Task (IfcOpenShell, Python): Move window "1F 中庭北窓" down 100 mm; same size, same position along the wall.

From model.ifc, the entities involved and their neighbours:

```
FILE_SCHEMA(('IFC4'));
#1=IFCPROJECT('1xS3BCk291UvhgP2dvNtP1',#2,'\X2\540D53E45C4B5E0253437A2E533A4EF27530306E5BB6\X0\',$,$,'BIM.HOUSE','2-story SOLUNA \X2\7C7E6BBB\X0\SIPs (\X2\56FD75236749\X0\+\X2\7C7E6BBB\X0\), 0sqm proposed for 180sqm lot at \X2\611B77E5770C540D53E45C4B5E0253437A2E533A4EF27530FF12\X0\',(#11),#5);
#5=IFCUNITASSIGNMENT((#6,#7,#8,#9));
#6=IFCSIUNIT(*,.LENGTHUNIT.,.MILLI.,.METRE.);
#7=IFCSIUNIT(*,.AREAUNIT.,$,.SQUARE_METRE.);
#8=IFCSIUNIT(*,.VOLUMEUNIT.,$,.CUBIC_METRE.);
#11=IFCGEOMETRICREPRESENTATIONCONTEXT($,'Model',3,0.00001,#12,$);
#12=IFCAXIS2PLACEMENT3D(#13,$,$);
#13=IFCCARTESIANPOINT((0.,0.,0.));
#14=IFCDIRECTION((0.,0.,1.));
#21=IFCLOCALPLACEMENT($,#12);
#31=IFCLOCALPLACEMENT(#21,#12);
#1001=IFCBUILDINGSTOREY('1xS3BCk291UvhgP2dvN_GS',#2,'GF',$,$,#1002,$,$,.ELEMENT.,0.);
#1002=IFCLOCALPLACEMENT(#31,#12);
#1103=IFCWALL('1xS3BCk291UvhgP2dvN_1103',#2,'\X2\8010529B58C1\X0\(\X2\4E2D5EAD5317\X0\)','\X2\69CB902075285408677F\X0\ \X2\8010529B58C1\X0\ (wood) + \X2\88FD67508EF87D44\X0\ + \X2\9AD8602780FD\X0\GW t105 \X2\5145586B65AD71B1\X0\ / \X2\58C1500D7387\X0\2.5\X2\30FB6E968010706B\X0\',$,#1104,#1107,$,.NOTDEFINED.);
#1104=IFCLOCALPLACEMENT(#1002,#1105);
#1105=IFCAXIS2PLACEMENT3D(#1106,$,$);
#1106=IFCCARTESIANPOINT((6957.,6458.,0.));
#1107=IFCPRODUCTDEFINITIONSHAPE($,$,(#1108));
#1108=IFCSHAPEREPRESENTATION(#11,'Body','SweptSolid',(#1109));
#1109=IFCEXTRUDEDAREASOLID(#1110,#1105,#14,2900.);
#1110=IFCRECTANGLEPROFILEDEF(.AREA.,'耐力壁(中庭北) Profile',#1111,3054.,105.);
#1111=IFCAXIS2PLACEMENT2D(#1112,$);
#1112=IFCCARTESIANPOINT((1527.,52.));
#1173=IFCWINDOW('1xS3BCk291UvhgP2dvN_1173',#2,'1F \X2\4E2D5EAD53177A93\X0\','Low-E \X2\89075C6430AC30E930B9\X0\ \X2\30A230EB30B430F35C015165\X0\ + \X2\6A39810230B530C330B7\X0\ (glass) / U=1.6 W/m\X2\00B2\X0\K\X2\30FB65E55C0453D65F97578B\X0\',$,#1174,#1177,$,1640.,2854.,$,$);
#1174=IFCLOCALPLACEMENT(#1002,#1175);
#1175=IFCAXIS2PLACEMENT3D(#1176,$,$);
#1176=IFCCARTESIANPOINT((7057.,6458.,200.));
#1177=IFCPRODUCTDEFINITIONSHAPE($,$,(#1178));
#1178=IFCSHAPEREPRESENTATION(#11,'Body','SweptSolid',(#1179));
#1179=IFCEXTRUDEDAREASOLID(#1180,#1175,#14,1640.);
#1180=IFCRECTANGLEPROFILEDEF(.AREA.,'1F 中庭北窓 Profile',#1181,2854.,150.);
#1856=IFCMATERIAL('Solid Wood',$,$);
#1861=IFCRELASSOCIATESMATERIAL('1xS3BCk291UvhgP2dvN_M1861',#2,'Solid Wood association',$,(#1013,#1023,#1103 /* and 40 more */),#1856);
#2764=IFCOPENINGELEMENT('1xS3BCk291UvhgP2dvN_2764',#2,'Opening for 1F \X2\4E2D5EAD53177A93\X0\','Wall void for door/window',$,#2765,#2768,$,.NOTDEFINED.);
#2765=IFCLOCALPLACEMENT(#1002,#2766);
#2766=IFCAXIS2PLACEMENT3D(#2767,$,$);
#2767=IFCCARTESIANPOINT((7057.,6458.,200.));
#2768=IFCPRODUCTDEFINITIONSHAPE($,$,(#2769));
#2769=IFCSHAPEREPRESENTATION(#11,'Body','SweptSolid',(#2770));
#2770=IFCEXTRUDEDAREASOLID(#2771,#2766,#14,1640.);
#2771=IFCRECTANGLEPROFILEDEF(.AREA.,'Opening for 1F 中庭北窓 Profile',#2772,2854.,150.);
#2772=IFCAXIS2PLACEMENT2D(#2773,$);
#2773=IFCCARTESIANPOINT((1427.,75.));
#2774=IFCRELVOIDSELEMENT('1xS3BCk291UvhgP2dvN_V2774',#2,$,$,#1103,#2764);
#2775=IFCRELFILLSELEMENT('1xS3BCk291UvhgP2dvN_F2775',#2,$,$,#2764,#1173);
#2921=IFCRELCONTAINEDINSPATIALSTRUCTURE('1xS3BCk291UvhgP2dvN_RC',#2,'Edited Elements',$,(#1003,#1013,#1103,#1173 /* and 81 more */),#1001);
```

```python
import numpy as np
import ifcopenshell
import ifcopenshell.api.geometry
import ifcopenshell.util.placement
import ifcopenshell.util.unit

model = ifcopenshell.open("model.ifc")
unit_scale = ifcopenshell.util.unit.calculate_unit_scale(model)

window = model.by_guid("1xS3BCk291UvhgP2dvN_1173")
opening = window.FillsVoids[0].RelatingOpeningElement
dz = -0.1 / unit_scale

shift = np.array([0.0, 0.0, dz])
# The window is not placed relative to its opening, so move both.
for product in (opening, window):
    matrix = ifcopenshell.util.placement.get_local_placement(product.ObjectPlacement)
    matrix[:3, 3] += shift
    ifcopenshell.api.geometry.edit_object_placement(model, product=product, matrix=matrix, is_si=False)

print(f"moved by {dz * unit_scale:+.3f} m")

model.write("model_updated.ifc")
```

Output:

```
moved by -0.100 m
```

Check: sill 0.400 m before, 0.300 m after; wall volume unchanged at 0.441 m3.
